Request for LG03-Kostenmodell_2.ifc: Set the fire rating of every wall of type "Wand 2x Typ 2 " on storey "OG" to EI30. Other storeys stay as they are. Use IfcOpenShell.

First a look at what the model holds.

```python
import ifcopenshell
import ifcopenshell.util.element

model = ifcopenshell.open("LG03-Kostenmodell_2.ifc")
print(model.schema)
storey = next(s for s in model.by_type("IfcBuildingStorey") if s.Name == "OG")
walls = [e for e in ifcopenshell.util.element.get_decomposition(storey) if e.is_a("IfcWall")]
seen = {}
for e in walls:
    element_type = ifcopenshell.util.element.get_type(e)
    key = (element_type.Name if element_type != e and element_type else None, ifcopenshell.util.element.get_pset(e, "Pset_WallCommon", "FireRating"))
    seen[key] = seen.get(key, 0) + 1
for (name, value), count in sorted(seen.items(), key=str):
    print(count, "x", name, "|", value)
```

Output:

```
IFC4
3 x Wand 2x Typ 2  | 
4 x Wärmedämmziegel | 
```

```python
import ifcopenshell
import ifcopenshell.api.pset
import ifcopenshell.util.element

model = ifcopenshell.open("LG03-Kostenmodell_2.ifc")

storey = next(s for s in model.by_type("IfcBuildingStorey") if s.Name == "OG")
walls = [e for e in ifcopenshell.util.element.get_decomposition(storey) if e.is_a("IfcWall")]

count = 0
for e in walls:
    element_type = ifcopenshell.util.element.get_type(e)
    if element_type in (None, e) or element_type.Name != "Wand 2x Typ 2 ":
        continue
    # add_pset returns the element's existing set when there is one.
    pset = ifcopenshell.api.pset.add_pset(model, product=e, name="Pset_WallCommon")
    ifcopenshell.api.pset.edit_pset(model, pset=pset, properties={"FireRating": "EI30"})
    count += 1

print(count, "walls updated")

model.write("LG03-Kostenmodell_2_edited.ifc")
```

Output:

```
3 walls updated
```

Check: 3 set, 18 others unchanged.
